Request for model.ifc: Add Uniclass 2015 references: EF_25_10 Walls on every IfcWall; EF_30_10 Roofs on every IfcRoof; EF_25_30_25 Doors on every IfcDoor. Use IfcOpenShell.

First a look at what the model holds.

```python
import ifcopenshell

model = ifcopenshell.open("model.ifc")
print(model.schema)
print("classifications:", [c.Name for c in model.by_type("IfcClassification")])
for ifc_class in ("IfcDoor", "IfcRoof", "IfcStair", "IfcWall", "IfcWindow"):
    print(ifc_class, len(model.by_type(ifc_class)))
```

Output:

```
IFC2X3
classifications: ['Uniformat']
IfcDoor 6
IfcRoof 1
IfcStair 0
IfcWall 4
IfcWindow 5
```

```python
import ifcopenshell
import ifcopenshell.api.classification

model = ifcopenshell.open("model.ifc")

# IFC2X3 requires Source and Edition and has no link from the project to the system.
system = model.create_entity("IfcClassification", Source="NBS", Edition="2015", Name="Uniclass 2015")

codes = {
    "IfcWall": ("EF_25_10", "Walls"),
    "IfcRoof": ("EF_30_10", "Roofs"),
    "IfcDoor": ("EF_25_30_25", "Doors"),
}
for ifc_class, (code, name) in codes.items():
    products = model.by_type(ifc_class)
    ifcopenshell.api.classification.add_reference(
        model, products=products, classification=system, identification=code, name=name
    )
    print(code, len(products))

model.write("model_rev.ifc")
```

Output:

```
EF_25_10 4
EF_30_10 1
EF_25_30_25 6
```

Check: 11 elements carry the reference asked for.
